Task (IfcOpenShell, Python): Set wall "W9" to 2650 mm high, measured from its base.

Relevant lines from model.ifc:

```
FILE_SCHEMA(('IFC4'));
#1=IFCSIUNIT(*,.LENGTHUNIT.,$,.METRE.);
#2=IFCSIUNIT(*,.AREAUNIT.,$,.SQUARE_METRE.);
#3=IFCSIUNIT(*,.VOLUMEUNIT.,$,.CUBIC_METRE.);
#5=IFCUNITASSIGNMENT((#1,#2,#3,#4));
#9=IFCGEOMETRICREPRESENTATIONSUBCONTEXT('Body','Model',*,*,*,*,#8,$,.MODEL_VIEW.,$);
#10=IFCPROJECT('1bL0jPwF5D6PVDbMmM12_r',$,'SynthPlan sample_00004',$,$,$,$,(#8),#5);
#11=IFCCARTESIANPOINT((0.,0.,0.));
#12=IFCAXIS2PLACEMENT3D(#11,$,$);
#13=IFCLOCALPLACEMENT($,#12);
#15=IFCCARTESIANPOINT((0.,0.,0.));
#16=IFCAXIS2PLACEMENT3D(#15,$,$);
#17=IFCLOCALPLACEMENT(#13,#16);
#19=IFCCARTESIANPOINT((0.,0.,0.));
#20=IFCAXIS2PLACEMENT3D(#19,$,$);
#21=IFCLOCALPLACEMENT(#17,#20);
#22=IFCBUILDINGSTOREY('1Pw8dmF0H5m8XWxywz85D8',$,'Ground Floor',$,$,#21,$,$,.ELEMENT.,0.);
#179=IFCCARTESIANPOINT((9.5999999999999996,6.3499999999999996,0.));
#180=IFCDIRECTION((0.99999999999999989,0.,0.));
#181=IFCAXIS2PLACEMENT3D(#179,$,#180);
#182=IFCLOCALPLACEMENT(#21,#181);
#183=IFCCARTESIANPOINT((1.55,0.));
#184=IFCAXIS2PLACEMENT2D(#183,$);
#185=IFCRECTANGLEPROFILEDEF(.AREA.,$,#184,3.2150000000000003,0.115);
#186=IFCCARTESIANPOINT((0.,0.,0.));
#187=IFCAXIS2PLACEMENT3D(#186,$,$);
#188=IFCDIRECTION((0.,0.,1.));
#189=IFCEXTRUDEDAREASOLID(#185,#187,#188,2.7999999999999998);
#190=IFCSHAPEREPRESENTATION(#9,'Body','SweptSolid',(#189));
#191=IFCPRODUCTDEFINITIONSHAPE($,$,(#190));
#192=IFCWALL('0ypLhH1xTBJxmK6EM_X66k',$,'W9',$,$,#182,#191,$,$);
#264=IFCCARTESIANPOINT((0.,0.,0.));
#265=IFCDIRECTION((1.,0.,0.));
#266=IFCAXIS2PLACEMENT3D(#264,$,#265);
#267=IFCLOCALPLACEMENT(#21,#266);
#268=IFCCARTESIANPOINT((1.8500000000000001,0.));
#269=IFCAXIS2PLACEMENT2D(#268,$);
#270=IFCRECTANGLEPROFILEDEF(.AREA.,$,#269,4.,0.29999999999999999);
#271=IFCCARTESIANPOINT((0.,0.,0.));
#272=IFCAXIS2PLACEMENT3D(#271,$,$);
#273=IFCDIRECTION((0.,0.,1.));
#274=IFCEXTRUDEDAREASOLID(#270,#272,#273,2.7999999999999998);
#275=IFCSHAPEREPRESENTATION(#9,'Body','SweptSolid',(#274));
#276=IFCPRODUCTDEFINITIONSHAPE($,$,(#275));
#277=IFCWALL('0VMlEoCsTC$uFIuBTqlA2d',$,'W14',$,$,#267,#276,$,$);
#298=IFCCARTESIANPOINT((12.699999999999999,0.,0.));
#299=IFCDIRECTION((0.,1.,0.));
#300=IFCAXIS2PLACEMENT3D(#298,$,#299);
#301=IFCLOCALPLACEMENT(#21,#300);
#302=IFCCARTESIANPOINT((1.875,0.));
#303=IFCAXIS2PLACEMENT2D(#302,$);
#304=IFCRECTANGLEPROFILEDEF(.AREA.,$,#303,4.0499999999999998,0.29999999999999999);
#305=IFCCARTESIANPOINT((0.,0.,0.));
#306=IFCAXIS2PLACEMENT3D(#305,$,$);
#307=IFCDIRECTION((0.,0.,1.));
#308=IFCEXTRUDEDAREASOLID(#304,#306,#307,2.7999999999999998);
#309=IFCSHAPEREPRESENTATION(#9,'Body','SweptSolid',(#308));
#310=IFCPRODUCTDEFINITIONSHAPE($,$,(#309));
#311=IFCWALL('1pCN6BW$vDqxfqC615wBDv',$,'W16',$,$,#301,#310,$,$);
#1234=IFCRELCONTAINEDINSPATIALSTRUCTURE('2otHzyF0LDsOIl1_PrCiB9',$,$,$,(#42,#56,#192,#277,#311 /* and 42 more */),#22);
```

```python
import ifcopenshell
import ifcopenshell.geom
import ifcopenshell.util.representation
import ifcopenshell.util.shape
import ifcopenshell.util.unit

model = ifcopenshell.open("model.ifc")
unit_scale = ifcopenshell.util.unit.calculate_unit_scale(model)
settings = ifcopenshell.geom.settings()


def volume(element):
    """Net volume in cubic metres, openings subtracted."""
    shape = ifcopenshell.geom.create_shape(settings, element)
    return ifcopenshell.util.shape.get_volume(shape.geometry)


wall = model.by_id(192)
before = volume(wall)

body = ifcopenshell.util.representation.get_representation(wall, "Model", "Body")
solid = body.Items[0]
old_height = solid.Depth
solid.Depth = 2.65 / unit_scale
after = volume(wall)

print(f"height {old_height:g} -> {solid.Depth:g}, volume {before:.3f} -> {after:.3f} m3")

model.write("model-out.ifc")
```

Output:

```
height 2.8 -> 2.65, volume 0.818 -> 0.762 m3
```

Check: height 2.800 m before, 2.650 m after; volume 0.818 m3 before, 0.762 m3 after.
